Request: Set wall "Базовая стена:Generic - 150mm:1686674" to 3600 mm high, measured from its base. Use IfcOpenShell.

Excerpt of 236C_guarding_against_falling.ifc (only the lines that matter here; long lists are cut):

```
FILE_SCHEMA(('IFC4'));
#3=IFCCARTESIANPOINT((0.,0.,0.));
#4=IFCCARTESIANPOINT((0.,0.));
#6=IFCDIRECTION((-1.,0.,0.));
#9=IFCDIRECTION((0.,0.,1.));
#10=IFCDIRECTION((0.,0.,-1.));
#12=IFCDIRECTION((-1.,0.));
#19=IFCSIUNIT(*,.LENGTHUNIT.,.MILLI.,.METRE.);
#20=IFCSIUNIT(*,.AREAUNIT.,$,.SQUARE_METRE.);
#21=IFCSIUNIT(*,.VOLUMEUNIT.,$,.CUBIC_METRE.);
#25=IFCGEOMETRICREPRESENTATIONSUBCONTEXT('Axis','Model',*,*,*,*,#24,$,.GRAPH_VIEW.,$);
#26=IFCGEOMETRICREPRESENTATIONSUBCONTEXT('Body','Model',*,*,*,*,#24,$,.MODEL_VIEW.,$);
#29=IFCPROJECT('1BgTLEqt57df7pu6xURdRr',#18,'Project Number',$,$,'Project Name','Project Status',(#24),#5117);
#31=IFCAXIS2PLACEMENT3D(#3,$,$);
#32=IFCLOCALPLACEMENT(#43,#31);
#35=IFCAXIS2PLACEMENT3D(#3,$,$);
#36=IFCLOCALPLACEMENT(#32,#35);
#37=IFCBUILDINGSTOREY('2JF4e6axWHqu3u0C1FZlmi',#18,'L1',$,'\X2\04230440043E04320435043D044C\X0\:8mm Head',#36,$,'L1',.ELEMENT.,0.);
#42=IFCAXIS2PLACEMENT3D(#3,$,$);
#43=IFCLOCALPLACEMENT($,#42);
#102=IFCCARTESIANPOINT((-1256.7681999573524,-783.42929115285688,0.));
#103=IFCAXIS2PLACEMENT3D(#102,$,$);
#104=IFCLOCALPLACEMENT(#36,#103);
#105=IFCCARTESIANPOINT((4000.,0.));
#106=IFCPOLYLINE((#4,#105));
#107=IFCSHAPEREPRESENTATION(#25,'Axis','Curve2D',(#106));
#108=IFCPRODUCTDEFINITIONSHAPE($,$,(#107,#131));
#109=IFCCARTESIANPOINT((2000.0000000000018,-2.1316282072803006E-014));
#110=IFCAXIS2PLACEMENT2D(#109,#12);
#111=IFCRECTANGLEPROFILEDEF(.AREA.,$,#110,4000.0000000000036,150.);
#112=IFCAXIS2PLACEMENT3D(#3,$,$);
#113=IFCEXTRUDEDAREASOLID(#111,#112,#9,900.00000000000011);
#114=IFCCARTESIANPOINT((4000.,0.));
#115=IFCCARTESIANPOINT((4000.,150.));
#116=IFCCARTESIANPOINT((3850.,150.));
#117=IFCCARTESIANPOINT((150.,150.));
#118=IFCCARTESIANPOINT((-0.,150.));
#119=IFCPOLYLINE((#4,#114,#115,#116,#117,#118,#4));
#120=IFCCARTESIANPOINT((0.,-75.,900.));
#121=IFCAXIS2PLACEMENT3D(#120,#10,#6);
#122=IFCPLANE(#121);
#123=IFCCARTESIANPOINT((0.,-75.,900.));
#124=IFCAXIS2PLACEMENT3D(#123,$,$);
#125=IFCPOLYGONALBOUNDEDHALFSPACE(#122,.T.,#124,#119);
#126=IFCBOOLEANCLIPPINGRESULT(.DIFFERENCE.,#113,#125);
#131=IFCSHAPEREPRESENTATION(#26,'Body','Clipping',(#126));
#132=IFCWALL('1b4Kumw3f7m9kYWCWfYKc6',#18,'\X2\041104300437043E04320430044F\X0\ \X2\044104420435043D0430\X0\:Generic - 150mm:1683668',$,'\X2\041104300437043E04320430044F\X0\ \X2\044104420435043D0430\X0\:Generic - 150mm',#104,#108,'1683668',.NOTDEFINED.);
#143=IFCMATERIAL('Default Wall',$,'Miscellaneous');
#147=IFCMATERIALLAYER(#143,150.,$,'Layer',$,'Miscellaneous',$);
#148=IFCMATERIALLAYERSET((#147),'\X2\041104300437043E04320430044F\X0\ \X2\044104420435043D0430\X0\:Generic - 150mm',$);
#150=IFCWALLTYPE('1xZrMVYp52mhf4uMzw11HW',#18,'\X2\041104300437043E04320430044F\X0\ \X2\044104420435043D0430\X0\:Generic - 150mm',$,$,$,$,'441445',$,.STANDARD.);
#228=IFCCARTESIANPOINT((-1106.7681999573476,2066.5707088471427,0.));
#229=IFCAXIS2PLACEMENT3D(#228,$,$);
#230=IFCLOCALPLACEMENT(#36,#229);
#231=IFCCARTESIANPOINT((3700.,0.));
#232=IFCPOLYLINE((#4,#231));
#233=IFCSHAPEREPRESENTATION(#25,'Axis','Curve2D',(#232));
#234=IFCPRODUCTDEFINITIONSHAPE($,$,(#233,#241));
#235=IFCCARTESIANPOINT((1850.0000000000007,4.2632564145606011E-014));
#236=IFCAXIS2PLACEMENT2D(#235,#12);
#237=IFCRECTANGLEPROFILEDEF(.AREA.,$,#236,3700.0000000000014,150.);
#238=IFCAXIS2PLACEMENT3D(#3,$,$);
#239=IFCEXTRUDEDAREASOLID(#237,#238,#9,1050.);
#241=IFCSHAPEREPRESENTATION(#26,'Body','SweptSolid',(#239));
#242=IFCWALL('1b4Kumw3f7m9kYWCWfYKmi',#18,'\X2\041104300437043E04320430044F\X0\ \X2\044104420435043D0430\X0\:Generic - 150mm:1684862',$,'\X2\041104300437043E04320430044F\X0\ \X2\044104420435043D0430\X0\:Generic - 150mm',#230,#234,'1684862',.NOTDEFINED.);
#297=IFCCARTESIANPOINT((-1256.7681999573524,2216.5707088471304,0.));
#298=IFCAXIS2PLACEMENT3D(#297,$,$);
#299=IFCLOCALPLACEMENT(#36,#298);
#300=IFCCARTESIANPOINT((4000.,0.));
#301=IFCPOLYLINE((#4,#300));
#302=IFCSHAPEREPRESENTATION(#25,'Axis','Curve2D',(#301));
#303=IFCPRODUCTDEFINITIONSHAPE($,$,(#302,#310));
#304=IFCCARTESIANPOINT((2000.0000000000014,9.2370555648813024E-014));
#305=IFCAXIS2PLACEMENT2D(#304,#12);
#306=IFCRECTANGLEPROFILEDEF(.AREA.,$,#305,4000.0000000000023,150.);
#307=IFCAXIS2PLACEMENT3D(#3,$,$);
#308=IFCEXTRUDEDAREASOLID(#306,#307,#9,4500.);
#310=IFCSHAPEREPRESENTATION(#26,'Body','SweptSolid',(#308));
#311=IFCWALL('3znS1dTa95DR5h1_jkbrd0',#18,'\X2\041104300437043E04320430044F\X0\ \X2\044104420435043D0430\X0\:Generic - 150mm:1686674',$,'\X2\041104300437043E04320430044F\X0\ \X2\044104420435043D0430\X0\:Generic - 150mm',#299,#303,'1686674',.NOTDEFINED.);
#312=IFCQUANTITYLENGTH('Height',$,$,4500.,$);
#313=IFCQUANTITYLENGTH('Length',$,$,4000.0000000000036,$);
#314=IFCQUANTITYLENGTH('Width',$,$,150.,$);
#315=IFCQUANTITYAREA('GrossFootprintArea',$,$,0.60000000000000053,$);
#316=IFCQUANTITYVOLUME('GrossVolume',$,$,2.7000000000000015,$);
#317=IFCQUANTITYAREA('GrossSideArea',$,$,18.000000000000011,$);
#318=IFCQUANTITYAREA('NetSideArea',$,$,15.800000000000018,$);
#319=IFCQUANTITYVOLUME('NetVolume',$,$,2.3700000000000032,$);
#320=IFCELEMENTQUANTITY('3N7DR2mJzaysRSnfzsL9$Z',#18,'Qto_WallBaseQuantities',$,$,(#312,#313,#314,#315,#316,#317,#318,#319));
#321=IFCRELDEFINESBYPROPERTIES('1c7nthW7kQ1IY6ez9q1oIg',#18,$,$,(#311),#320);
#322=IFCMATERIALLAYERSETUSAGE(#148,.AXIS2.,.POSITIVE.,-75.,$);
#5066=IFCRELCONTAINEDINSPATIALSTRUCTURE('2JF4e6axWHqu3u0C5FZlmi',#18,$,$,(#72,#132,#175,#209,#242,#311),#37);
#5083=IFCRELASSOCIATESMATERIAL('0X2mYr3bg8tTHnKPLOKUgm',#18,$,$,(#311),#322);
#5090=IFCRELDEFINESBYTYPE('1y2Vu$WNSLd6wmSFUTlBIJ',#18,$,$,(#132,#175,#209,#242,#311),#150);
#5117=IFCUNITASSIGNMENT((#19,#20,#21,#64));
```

```python
import ifcopenshell
import ifcopenshell.api.pset
import ifcopenshell.geom
import ifcopenshell.util.element
import ifcopenshell.util.representation
import ifcopenshell.util.shape
import ifcopenshell.util.unit

model = ifcopenshell.open("236C_guarding_against_falling.ifc")
unit_scale = ifcopenshell.util.unit.calculate_unit_scale(model)
area_scale = ifcopenshell.util.unit.calculate_unit_scale(model, "AREAUNIT")
volume_scale = ifcopenshell.util.unit.calculate_unit_scale(model, "VOLUMEUNIT")
settings = ifcopenshell.geom.settings()


def volume(element):
    """Net volume in cubic metres, openings subtracted."""
    shape = ifcopenshell.geom.create_shape(settings, element)
    return ifcopenshell.util.shape.get_volume(shape.geometry)


wall = model.by_id(311)
before = volume(wall)

body = ifcopenshell.util.representation.get_representation(wall, "Model", "Body")
solid = body.Items[0]
old_height = solid.Depth
solid.Depth = 3.6 / unit_scale
after = volume(wall)
thickness = 0.15  # wall thickness in metres

# Update the stored height, areas and volumes.
qto = model.by_id(ifcopenshell.util.element.get_pset(wall, "Qto_WallBaseQuantities", should_inherit=False)["id"])
ifcopenshell.api.pset.edit_qto(model, qto=qto, properties={
    "Height": solid.Depth,
    "GrossVolume": ifcopenshell.util.element.get_pset(wall, "Qto_WallBaseQuantities", "GrossVolume") * solid.Depth / old_height,
    "GrossSideArea": ifcopenshell.util.element.get_pset(wall, "Qto_WallBaseQuantities", "GrossSideArea") * solid.Depth / old_height,
    "NetSideArea": after / thickness / area_scale,
    "NetVolume": after / volume_scale,
})

print(f"height {old_height:g} -> {solid.Depth:g}, volume {before:.3f} -> {after:.3f} m3")

model.write("236C_guarding_against_falling-out.ifc")
```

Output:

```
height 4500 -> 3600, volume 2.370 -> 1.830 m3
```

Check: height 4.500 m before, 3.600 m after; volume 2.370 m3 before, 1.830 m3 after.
